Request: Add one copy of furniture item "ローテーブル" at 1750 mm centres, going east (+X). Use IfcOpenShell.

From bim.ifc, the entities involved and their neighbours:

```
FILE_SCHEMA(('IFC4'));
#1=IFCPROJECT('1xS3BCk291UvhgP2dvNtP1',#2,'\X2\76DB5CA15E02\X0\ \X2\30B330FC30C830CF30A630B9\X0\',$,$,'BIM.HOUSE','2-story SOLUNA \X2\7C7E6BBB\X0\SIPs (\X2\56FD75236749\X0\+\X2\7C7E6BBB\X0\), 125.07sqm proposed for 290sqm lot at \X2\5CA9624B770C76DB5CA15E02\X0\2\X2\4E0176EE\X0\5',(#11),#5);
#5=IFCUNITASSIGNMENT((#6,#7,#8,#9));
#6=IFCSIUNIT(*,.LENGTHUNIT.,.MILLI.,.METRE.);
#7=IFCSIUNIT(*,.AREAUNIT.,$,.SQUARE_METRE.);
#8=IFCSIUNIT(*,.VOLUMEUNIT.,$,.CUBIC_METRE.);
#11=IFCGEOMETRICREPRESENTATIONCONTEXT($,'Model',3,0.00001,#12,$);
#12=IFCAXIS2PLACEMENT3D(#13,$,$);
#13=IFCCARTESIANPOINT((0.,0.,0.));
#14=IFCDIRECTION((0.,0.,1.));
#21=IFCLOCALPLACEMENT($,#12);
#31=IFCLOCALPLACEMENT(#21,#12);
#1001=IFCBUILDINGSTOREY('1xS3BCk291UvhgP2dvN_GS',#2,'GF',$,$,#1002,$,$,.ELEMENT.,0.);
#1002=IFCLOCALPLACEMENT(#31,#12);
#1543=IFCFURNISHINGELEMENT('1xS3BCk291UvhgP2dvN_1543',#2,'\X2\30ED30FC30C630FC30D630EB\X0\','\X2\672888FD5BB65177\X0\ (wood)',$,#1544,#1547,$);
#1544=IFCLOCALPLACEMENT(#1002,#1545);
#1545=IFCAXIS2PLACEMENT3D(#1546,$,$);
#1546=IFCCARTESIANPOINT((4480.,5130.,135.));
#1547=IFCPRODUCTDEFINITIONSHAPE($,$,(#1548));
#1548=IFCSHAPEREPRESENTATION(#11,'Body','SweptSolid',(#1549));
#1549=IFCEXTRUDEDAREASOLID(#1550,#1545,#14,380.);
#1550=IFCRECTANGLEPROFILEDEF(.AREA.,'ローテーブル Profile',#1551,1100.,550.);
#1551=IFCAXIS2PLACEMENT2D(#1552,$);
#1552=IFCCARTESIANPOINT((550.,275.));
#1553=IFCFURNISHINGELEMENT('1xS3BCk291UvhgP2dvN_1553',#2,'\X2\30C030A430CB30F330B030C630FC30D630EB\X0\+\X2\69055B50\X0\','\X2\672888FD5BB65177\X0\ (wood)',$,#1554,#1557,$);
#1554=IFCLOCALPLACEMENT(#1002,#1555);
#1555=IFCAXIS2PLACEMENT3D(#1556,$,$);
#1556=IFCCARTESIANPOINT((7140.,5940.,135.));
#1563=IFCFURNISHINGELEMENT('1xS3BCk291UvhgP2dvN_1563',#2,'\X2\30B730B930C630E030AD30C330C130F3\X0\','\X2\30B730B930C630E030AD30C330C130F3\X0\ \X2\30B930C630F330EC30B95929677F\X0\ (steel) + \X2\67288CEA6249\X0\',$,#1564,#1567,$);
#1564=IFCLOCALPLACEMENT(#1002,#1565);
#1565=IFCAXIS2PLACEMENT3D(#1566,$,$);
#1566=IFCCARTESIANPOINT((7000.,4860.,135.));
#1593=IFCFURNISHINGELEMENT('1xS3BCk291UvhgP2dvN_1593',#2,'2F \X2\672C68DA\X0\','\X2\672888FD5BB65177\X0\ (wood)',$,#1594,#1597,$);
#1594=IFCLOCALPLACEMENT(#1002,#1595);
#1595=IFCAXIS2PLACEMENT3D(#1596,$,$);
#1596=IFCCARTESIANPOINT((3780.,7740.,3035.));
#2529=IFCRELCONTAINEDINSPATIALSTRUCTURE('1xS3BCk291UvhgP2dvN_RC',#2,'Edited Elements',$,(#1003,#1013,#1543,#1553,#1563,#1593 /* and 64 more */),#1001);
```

```python
import numpy as np
import ifcopenshell
import ifcopenshell.api.geometry
import ifcopenshell.api.root
import ifcopenshell.util.element
import ifcopenshell.util.placement

model = ifcopenshell.open("bim.ifc")


def reuse_history(source, copy):
    """copy_class also copies each property set's owner history, people and application; keep the originals."""
    for rel in copy.IsDefinedBy:
        if rel.is_a("IfcRelDefinesByProperties") and (history := rel.RelatingPropertyDefinition.OwnerHistory):
            rel.RelatingPropertyDefinition.OwnerHistory = source.OwnerHistory
            ifcopenshell.util.element.remove_deep2(model, history)


source = model.by_id(1543)
base = ifcopenshell.util.placement.get_local_placement(source.ObjectPlacement)
step = np.array([1.0, 0.0, 0.0]) * 1750.0

for i in range(1, 2):
    copy = ifcopenshell.api.root.copy_class(model, product=source)
    copy.Representation = ifcopenshell.util.element.copy_deep(
        model, source.Representation, exclude=["IfcGeometricRepresentationContext", "IfcRepresentationMap"]
    )
    reuse_history(source, copy)
    matrix = base.copy()
    matrix[:3, 3] += i * step
    print("added at", matrix[:3, 3].round(3) + 0.0)
    ifcopenshell.api.geometry.edit_object_placement(model, product=copy, matrix=matrix, is_si=False)

model.write("bim_edited.ifc")
```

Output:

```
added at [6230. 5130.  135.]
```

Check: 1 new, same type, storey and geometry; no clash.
